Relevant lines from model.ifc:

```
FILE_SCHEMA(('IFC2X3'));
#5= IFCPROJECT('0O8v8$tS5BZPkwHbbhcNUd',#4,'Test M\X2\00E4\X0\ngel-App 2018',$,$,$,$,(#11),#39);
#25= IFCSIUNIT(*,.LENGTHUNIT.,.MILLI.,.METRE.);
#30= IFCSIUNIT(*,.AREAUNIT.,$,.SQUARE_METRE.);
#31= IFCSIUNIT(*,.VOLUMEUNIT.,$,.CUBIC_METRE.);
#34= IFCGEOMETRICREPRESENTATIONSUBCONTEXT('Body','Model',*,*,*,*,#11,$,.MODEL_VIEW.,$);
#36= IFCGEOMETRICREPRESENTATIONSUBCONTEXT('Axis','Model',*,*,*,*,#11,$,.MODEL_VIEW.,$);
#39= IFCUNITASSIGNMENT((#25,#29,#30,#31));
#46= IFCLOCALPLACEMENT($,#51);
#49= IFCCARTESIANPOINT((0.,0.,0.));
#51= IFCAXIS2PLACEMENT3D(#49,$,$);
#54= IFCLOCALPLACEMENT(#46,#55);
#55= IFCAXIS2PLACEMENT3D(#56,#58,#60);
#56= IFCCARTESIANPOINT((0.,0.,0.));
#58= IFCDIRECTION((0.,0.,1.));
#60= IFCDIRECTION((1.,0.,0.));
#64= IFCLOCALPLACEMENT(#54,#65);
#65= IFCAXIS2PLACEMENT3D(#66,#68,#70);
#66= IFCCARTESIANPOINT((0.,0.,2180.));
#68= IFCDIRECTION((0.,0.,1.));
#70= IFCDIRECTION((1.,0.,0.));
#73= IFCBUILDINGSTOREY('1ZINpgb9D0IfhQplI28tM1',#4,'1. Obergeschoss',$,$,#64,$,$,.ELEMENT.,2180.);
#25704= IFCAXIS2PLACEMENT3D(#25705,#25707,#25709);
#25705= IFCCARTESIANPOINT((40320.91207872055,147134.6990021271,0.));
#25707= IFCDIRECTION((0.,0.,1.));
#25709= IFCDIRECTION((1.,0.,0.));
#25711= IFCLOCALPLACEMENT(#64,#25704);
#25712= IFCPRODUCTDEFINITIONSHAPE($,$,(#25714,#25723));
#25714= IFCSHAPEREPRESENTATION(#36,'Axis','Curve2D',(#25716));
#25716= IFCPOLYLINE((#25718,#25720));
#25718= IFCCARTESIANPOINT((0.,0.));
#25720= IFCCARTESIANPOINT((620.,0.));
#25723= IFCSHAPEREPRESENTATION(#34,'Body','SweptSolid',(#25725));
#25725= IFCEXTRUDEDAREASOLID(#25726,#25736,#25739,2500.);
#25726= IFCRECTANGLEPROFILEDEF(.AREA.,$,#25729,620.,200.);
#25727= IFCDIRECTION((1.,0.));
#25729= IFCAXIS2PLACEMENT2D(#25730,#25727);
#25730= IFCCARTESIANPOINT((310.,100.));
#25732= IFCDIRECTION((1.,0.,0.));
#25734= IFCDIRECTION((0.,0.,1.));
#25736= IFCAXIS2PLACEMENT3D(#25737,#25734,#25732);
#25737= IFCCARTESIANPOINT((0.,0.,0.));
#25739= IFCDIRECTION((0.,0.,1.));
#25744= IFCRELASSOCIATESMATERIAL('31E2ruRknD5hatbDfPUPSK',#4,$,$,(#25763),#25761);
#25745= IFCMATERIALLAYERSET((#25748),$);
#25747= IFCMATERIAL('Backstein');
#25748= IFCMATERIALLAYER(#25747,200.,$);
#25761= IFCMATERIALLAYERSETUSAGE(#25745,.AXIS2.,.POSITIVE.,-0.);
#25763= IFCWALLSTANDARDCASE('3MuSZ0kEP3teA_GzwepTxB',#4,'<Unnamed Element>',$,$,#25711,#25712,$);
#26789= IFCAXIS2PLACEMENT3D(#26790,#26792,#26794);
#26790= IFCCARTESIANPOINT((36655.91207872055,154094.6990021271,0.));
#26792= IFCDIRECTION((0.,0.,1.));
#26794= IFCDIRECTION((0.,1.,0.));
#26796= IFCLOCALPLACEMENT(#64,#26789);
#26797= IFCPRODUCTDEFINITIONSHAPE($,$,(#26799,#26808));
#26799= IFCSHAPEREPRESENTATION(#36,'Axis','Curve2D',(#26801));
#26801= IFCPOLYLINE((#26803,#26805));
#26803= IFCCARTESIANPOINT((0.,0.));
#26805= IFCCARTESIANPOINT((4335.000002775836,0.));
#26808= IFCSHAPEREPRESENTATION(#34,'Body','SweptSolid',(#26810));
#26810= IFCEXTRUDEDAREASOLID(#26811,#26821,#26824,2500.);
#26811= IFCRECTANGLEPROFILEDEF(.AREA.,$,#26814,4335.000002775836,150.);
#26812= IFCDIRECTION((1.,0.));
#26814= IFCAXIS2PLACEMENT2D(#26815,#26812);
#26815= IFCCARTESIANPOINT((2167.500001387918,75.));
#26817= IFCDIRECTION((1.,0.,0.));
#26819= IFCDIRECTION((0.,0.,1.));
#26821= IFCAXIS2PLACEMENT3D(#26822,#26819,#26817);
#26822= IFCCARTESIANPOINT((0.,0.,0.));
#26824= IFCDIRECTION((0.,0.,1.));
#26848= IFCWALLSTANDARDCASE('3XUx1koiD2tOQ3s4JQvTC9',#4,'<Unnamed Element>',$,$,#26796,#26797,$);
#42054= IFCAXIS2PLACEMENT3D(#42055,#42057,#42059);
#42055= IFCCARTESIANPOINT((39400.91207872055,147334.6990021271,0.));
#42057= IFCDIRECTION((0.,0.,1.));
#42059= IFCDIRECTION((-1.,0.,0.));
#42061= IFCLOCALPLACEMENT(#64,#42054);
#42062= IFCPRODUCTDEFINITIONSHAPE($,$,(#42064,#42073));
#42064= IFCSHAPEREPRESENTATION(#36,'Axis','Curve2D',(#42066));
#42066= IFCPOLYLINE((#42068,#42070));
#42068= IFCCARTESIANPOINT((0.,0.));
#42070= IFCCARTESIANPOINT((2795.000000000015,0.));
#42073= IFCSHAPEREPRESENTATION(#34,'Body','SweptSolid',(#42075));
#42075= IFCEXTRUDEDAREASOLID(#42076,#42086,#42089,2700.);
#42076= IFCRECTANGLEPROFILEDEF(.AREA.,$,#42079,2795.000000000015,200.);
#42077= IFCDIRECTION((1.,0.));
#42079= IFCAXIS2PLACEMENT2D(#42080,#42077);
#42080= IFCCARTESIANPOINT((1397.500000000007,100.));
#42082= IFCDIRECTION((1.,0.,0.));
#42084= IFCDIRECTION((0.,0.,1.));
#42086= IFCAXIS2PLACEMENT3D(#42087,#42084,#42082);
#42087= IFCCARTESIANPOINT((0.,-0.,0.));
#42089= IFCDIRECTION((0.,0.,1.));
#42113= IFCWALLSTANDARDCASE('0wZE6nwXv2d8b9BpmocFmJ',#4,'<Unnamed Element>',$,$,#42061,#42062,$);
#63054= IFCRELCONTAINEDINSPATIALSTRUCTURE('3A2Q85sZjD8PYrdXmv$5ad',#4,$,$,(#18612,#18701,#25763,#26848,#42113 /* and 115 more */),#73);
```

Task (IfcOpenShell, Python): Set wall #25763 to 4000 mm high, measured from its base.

```python
import ifcopenshell
import ifcopenshell.geom
import ifcopenshell.util.representation
import ifcopenshell.util.shape
import ifcopenshell.util.unit

model = ifcopenshell.open("model.ifc")
unit_scale = ifcopenshell.util.unit.calculate_unit_scale(model)
settings = ifcopenshell.geom.settings()


def volume(element):
    """Net volume in cubic metres, openings subtracted."""
    shape = ifcopenshell.geom.create_shape(settings, element)
    return ifcopenshell.util.shape.get_volume(shape.geometry)


wall = model.by_id(25763)
before = volume(wall)

body = ifcopenshell.util.representation.get_representation(wall, "Model", "Body")
solid = body.Items[0]
old_height = solid.Depth
solid.Depth = 4 / unit_scale
after = volume(wall)

print(f"height {old_height:g} -> {solid.Depth:g}, volume {before:.3f} -> {after:.3f} m3")

model.write("model_v2.ifc")
```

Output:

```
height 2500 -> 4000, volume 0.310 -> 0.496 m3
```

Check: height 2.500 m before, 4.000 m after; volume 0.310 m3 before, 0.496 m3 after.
